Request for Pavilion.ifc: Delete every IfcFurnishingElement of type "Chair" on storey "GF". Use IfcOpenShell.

First a look at what the model holds.

```python
import ifcopenshell
import ifcopenshell.util.element

model = ifcopenshell.open("Pavilion.ifc")
print(model.schema)
storey = next(s for s in model.by_type("IfcBuildingStorey") if s.Name == "GF")
furniture = [e for e in ifcopenshell.util.element.get_decomposition(storey) if e.is_a("IfcFurnishingElement")]
seen = {}
for e in furniture:
    element_type = ifcopenshell.util.element.get_type(e)
    name = element_type.Name if element_type not in (None, e) else None
    seen[name] = seen.get(name, 0) + 1
for name, count in sorted(seen.items(), key=str):
    print(count, "x", name)
```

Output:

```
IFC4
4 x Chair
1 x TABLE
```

```python
import ifcopenshell
import ifcopenshell.api.root
import ifcopenshell.util.element

model = ifcopenshell.open("Pavilion.ifc")

storey = next(s for s in model.by_type("IfcBuildingStorey") if s.Name == "GF")
furniture = [e for e in ifcopenshell.util.element.get_decomposition(storey) if e.is_a("IfcFurnishingElement")]
targets = [e for e in furniture if (t := ifcopenshell.util.element.get_type(e)) not in (None, e) and t.Name == "Chair"]

for e in targets:
    ifcopenshell.api.root.remove_product(model, product=e)
print(len(targets), "removed")

model.write("Pavilion_edited.ifc")
```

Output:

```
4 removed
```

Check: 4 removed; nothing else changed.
